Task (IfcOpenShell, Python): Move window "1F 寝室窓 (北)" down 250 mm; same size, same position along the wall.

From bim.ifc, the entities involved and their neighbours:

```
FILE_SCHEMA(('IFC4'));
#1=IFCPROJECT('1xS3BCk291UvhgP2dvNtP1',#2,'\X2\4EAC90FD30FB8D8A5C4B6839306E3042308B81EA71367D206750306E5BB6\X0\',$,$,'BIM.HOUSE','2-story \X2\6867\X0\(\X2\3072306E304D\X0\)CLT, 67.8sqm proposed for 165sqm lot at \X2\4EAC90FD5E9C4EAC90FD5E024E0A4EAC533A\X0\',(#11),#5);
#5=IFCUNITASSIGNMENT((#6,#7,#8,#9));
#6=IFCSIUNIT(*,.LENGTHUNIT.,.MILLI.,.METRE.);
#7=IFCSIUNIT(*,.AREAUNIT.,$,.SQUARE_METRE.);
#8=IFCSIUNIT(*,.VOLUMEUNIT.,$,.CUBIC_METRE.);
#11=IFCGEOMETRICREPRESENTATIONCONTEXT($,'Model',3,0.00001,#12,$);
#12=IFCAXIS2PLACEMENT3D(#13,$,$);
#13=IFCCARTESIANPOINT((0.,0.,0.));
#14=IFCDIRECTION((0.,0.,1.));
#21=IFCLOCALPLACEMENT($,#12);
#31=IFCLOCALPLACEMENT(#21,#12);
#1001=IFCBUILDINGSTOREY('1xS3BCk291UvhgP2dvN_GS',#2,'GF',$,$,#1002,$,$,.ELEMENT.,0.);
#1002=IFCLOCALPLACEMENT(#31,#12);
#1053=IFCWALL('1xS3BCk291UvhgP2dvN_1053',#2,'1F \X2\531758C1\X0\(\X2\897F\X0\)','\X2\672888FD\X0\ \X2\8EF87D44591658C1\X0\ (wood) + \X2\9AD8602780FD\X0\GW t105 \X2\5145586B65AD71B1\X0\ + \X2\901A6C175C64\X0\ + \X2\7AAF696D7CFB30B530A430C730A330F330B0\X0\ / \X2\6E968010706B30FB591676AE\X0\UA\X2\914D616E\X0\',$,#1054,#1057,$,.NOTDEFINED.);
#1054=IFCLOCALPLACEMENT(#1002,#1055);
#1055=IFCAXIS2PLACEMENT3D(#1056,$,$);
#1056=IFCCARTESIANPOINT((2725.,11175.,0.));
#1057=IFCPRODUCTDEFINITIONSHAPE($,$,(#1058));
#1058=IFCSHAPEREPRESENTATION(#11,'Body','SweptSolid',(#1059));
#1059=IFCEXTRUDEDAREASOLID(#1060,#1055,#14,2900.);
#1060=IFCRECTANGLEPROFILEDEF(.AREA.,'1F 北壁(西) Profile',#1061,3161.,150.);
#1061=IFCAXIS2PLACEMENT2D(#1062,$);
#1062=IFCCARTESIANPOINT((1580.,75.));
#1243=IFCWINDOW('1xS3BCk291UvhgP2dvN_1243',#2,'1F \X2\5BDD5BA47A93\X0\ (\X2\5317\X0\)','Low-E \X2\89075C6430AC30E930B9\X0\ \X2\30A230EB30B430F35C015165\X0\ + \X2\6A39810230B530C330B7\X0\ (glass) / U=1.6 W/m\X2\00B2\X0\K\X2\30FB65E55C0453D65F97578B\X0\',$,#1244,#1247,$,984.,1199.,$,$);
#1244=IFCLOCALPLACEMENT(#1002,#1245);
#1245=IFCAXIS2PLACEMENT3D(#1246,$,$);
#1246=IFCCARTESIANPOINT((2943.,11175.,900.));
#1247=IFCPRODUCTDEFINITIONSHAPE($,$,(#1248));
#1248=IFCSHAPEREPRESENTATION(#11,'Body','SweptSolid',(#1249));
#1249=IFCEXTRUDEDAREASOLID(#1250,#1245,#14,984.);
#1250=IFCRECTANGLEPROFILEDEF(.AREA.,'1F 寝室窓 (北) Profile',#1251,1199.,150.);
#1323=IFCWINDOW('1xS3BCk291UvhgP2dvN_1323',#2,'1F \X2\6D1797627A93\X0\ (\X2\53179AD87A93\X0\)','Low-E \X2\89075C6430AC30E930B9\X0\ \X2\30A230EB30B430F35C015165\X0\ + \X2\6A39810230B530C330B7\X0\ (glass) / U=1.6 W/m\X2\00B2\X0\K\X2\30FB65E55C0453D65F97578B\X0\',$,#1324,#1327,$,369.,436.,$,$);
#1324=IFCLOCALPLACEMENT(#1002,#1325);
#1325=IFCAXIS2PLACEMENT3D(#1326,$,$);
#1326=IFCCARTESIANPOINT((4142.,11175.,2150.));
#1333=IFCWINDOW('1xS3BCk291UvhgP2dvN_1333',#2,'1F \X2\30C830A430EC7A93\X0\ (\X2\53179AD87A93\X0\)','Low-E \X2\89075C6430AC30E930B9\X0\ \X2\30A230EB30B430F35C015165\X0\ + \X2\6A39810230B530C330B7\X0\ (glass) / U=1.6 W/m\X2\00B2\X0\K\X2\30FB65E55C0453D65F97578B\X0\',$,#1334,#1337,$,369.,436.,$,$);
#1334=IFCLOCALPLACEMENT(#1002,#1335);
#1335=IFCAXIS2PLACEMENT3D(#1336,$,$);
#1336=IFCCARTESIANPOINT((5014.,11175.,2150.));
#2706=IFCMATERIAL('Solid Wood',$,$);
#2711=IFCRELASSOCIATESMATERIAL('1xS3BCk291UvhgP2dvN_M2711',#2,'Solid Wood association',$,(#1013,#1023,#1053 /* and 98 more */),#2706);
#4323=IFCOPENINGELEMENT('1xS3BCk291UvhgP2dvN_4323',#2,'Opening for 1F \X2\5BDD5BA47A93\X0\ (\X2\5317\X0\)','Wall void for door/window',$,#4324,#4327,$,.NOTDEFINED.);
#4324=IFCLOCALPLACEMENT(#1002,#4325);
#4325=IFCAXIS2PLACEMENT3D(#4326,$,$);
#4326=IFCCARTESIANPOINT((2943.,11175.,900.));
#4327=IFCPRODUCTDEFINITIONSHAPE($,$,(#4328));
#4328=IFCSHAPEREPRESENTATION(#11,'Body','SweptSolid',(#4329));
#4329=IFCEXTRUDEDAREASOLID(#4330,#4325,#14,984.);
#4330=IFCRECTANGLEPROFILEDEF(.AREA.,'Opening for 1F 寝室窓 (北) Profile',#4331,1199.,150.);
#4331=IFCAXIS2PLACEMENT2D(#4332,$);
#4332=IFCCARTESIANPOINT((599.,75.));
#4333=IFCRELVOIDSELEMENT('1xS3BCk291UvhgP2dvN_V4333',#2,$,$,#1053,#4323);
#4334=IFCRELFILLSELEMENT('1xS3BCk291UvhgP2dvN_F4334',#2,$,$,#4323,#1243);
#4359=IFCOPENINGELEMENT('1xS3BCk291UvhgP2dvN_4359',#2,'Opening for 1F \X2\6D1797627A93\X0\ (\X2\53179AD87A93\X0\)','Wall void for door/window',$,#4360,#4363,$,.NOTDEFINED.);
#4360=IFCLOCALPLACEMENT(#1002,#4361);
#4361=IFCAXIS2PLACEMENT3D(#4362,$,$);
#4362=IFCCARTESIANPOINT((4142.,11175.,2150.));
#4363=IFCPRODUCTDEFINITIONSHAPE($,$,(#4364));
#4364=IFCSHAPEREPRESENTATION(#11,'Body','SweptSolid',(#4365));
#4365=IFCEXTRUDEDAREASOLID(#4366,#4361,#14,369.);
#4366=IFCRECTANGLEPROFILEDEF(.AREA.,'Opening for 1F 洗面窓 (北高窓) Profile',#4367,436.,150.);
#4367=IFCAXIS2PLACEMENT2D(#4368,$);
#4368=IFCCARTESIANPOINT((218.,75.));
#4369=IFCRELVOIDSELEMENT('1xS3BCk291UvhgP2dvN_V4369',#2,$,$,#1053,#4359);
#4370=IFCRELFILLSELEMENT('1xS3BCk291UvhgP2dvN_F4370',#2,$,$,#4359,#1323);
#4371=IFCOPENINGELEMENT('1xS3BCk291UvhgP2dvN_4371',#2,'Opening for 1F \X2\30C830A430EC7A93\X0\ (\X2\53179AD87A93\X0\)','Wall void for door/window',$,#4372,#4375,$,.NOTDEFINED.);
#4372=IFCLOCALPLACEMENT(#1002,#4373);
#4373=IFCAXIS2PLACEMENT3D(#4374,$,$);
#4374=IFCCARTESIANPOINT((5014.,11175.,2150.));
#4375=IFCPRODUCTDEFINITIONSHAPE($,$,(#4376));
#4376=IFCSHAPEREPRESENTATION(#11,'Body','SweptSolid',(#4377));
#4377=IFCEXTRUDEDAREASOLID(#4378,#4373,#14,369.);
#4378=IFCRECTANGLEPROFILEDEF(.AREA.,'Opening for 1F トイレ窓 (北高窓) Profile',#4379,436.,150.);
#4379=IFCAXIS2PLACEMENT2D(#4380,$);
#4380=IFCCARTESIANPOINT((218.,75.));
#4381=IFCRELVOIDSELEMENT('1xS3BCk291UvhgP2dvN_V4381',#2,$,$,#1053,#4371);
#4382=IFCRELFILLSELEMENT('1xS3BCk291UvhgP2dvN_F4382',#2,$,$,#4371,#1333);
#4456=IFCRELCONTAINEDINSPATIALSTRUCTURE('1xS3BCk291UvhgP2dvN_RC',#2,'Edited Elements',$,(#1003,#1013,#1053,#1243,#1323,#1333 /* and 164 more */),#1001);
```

```python
import numpy as np
import ifcopenshell
import ifcopenshell.api.geometry
import ifcopenshell.util.placement
import ifcopenshell.util.unit

model = ifcopenshell.open("bim.ifc")
unit_scale = ifcopenshell.util.unit.calculate_unit_scale(model)

window = model.by_guid("1xS3BCk291UvhgP2dvN_1243")
opening = window.FillsVoids[0].RelatingOpeningElement
dz = -0.25 / unit_scale

shift = np.array([0.0, 0.0, dz])
# The window is not placed relative to its opening, so move both.
for product in (opening, window):
    matrix = ifcopenshell.util.placement.get_local_placement(product.ObjectPlacement)
    matrix[:3, 3] += shift
    ifcopenshell.api.geometry.edit_object_placement(model, product=product, matrix=matrix, is_si=False)

print(f"moved by {dz * unit_scale:+.3f} m")

model.write("bim-out.ifc")
```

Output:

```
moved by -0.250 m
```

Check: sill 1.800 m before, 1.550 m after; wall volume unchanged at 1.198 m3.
